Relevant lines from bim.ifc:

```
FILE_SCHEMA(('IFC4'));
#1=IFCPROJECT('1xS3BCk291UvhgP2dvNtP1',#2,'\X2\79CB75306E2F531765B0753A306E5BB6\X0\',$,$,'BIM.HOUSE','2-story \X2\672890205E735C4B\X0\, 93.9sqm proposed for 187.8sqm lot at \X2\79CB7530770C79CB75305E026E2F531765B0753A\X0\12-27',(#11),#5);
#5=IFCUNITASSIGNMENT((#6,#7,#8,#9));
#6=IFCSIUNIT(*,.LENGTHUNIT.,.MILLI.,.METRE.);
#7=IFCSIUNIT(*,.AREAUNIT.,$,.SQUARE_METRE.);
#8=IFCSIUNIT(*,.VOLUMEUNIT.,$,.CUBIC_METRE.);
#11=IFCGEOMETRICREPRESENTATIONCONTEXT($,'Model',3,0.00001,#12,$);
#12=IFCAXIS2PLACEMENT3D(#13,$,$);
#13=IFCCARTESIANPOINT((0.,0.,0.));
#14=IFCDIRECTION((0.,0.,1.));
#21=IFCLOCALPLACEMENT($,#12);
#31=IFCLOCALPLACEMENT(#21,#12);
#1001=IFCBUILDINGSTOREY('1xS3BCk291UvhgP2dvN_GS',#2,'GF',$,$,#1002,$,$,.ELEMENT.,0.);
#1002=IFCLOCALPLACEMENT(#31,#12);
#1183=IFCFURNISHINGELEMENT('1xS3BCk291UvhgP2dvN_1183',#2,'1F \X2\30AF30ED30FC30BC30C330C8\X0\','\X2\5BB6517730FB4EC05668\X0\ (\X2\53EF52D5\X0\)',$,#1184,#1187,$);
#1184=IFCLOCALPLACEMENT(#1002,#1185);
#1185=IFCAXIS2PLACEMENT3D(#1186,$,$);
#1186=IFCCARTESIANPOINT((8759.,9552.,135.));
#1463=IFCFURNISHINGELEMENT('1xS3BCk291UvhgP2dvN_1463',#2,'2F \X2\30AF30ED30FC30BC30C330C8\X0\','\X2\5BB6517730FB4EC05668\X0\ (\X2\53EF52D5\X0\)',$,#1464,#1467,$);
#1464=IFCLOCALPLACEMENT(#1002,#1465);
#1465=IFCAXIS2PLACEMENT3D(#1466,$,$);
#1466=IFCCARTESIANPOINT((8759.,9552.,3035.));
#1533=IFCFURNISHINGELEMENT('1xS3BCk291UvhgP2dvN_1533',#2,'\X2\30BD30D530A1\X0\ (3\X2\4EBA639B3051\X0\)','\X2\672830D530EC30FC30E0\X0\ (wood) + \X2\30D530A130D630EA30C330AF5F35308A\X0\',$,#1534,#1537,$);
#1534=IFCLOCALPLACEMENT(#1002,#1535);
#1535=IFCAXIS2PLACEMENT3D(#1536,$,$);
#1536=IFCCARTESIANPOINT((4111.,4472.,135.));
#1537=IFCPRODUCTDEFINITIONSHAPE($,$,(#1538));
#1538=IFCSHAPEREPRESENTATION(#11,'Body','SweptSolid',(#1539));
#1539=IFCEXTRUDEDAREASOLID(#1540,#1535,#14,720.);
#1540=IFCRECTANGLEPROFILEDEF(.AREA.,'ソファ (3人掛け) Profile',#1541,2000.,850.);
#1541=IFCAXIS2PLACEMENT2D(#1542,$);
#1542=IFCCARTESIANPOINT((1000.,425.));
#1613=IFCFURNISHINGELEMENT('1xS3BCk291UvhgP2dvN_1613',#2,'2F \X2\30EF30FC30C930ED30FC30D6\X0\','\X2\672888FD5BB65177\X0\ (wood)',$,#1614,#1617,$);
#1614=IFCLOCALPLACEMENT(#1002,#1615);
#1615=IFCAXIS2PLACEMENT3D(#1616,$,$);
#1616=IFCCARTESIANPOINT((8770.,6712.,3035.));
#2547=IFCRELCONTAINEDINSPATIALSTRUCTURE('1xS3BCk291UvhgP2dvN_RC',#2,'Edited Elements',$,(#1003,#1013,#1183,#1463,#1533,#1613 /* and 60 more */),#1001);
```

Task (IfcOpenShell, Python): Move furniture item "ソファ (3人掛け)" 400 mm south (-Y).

```python
import ifcopenshell
import ifcopenshell.api.geometry
import ifcopenshell.util.placement
import ifcopenshell.util.unit

model = ifcopenshell.open("bim.ifc")
unit_scale = ifcopenshell.util.unit.calculate_unit_scale(model)

item = model.by_id(1533)
matrix = ifcopenshell.util.placement.get_local_placement(item.ObjectPlacement)
matrix[1, 3] -= 0.4 / unit_scale
ifcopenshell.api.geometry.edit_object_placement(model, product=item, matrix=matrix, is_si=False)

print(ifcopenshell.util.placement.get_local_placement(item.ObjectPlacement).round(3) + 0.0)

model.write("bim-out.ifc")
```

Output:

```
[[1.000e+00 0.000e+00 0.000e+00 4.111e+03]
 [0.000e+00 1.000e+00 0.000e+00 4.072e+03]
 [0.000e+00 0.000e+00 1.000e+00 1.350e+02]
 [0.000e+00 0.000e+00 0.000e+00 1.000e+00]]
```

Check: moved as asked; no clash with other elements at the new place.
